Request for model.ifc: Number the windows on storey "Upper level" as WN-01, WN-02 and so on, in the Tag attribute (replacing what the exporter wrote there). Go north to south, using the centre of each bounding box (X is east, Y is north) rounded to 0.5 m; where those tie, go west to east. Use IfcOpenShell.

First a look at what the model holds.

```python
import ifcopenshell
import ifcopenshell.util.element
import ifcopenshell.util.placement

model = ifcopenshell.open("model.ifc")
print(model.schema)
storey = next(s for s in model.by_type("IfcBuildingStorey") if s.Name == "Upper level")
windows = [e for e in ifcopenshell.util.element.get_decomposition(storey) if e.is_a("IfcWindow")]
for e in sorted(windows, key=lambda e: e.id()):
    origin = ifcopenshell.util.placement.get_local_placement(e.ObjectPlacement)[:3, 3]
    print(e.id(), e.Tag, e.Name, origin.round(2) + 0.0, sep=" | ")
```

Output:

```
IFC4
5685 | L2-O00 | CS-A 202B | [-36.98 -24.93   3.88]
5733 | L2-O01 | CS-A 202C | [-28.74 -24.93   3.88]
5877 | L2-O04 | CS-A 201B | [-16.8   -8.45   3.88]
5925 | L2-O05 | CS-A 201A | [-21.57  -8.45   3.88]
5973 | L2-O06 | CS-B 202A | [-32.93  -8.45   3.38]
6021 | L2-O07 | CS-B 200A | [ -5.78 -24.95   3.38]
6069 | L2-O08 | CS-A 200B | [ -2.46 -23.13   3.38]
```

```python
import ifcopenshell
import ifcopenshell.geom
import ifcopenshell.util.element
import ifcopenshell.util.shape

model = ifcopenshell.open("model.ifc")
settings = ifcopenshell.geom.settings()
settings.set("use-world-coords", True)


def centre(element):
    shape = ifcopenshell.geom.create_shape(settings, element)
    return ifcopenshell.util.shape.get_bbox_centroid(shape.geometry)


storey = next(s for s in model.by_type("IfcBuildingStorey") if s.Name == "Upper level")
windows = [e for e in ifcopenshell.util.element.get_decomposition(storey) if e.is_a("IfcWindow")]

# Insertion points can sit at a corner or the storey origin, so sort by the geometry (in metres).
centres = {e: centre(e) for e in windows}
windows.sort(key=lambda e: (-round(centres[e][1] / 0.5), centres[e][0]))

for i, e in enumerate(windows, start=1):
    number = f"WN-{i:02d}"
    e.Tag = number
    print(e.id(), number)

model.write("model_rev.ifc")
```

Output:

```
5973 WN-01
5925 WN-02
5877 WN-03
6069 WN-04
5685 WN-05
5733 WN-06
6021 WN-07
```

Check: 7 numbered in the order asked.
